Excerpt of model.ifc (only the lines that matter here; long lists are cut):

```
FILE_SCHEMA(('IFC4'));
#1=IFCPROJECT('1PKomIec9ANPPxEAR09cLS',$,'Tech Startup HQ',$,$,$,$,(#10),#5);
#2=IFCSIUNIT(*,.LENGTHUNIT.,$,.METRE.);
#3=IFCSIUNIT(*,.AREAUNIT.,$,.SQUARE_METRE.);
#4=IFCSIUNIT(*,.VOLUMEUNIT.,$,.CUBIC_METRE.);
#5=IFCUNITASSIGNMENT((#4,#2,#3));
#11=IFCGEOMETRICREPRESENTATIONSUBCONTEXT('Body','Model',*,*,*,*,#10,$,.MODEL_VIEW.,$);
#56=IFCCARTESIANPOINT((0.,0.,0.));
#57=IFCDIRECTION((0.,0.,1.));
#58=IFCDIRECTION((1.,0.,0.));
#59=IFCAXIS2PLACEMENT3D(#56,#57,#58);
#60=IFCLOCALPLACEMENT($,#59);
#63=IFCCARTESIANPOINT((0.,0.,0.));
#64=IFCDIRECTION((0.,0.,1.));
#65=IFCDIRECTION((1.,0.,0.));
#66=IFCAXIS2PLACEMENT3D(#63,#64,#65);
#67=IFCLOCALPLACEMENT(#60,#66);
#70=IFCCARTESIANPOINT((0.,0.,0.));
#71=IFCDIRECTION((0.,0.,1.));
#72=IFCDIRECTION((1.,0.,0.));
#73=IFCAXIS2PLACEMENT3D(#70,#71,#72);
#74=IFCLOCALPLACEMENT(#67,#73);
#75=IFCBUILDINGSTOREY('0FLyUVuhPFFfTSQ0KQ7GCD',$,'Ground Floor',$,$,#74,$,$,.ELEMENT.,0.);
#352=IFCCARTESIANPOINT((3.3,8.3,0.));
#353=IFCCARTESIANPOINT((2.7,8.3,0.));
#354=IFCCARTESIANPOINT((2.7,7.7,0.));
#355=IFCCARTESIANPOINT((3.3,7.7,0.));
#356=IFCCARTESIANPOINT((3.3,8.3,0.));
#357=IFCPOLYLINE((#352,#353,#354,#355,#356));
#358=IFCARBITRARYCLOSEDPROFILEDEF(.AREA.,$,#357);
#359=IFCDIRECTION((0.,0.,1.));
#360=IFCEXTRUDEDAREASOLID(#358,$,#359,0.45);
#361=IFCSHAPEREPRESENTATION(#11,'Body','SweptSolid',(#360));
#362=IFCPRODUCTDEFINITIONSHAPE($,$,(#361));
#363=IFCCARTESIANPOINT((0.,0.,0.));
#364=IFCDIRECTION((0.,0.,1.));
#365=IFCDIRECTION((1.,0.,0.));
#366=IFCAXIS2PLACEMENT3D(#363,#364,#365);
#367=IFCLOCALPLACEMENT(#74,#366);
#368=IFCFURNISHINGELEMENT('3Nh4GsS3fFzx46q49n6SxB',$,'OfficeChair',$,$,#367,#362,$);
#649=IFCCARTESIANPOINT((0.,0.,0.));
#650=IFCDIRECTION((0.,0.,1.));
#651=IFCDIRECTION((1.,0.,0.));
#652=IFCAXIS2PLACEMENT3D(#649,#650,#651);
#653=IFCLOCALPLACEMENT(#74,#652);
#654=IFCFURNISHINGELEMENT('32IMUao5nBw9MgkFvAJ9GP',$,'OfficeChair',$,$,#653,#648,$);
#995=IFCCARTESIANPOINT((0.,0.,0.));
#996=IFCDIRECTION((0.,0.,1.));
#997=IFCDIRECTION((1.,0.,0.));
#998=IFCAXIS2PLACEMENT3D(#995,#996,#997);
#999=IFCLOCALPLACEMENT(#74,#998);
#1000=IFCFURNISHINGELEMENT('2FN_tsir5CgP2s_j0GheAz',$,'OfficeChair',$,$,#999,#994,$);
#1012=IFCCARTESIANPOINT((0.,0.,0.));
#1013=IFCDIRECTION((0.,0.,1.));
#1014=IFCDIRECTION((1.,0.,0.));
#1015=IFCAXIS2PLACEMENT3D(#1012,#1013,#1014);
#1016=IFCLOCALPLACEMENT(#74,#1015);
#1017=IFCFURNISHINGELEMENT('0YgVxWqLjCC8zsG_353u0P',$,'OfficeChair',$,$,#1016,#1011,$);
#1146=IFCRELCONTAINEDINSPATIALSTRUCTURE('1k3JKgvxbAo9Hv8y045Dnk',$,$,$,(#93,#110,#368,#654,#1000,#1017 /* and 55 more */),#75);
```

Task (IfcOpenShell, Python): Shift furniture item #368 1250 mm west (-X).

```python
import ifcopenshell
import ifcopenshell.api.geometry
import ifcopenshell.util.placement
import ifcopenshell.util.unit

model = ifcopenshell.open("model.ifc")
unit_scale = ifcopenshell.util.unit.calculate_unit_scale(model)

item = model.by_id(368)
matrix = ifcopenshell.util.placement.get_local_placement(item.ObjectPlacement)
matrix[0, 3] -= 1.25 / unit_scale
ifcopenshell.api.geometry.edit_object_placement(model, product=item, matrix=matrix, is_si=False)

print(ifcopenshell.util.placement.get_local_placement(item.ObjectPlacement).round(3) + 0.0)

model.write("model-out.ifc")
```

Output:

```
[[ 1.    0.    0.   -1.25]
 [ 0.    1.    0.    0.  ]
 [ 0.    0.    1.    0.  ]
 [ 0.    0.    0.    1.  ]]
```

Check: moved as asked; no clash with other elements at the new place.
